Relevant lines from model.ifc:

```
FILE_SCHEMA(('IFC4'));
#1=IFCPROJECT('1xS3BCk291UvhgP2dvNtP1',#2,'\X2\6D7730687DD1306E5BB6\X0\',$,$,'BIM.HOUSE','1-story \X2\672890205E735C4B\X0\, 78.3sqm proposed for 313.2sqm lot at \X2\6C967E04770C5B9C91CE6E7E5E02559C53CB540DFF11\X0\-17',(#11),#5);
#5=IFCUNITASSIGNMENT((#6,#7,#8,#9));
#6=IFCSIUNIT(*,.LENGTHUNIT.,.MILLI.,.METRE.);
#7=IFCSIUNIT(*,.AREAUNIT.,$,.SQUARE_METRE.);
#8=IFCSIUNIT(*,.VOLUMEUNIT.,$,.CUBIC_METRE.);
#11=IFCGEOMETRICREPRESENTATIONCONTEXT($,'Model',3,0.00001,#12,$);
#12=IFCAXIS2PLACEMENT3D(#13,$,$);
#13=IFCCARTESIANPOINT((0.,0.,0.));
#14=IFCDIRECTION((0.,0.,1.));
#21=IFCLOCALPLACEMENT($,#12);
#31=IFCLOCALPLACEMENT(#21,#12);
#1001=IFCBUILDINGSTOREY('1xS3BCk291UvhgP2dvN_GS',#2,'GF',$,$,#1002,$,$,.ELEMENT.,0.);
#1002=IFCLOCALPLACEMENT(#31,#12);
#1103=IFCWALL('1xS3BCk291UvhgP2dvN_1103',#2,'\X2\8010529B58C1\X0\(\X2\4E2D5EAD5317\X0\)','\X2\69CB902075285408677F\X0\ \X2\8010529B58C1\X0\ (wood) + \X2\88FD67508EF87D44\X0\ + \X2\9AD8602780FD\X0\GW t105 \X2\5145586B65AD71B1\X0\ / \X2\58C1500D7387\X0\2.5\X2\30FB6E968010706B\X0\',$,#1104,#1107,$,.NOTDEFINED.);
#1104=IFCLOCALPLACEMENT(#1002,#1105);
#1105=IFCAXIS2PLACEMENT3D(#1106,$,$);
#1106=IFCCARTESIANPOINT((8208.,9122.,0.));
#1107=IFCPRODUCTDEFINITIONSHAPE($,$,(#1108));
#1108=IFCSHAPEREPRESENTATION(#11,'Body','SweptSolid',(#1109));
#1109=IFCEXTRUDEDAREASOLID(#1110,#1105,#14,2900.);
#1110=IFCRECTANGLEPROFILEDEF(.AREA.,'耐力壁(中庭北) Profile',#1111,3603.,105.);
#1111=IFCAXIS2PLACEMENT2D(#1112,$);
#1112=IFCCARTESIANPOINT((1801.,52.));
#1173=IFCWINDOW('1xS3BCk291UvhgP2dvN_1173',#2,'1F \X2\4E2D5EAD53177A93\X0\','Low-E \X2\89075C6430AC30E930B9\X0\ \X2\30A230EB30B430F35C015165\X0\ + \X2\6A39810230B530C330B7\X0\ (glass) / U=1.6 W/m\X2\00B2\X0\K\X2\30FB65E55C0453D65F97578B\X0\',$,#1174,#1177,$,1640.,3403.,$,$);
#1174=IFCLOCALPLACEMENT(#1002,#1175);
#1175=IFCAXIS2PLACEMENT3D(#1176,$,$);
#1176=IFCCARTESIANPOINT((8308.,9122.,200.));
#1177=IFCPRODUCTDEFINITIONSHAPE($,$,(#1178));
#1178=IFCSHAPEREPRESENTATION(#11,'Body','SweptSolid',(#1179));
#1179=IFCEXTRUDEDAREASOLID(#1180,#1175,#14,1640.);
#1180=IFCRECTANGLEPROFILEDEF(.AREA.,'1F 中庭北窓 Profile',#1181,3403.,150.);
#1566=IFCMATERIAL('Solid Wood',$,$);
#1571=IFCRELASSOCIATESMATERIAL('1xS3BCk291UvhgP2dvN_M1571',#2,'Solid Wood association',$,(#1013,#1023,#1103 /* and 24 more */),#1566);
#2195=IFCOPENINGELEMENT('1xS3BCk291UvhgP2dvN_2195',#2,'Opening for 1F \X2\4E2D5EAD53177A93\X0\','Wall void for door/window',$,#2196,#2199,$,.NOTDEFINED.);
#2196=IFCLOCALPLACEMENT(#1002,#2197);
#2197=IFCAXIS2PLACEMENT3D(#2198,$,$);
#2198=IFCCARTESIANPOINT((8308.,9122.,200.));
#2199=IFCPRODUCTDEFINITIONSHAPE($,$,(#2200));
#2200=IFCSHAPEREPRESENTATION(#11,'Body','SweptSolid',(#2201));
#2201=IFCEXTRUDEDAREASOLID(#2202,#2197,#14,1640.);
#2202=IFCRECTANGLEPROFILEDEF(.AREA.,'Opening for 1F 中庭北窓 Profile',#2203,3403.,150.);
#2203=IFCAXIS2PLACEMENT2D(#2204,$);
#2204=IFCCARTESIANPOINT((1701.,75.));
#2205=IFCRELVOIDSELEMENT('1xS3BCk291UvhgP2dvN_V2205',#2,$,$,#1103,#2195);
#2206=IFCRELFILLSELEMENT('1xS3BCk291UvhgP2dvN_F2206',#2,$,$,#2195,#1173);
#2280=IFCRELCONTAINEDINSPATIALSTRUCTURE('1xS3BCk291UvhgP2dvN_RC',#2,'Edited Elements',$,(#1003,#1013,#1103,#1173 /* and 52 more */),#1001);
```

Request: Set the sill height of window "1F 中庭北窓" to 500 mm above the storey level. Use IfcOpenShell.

```python
import numpy as np
import ifcopenshell
import ifcopenshell.api.geometry
import ifcopenshell.geom
import ifcopenshell.util.element
import ifcopenshell.util.placement
import ifcopenshell.util.shape
import ifcopenshell.util.unit

model = ifcopenshell.open("model.ifc")
unit_scale = ifcopenshell.util.unit.calculate_unit_scale(model)

window = model.by_id(1173)
opening = window.FillsVoids[0].RelatingOpeningElement
storey = ifcopenshell.util.element.get_container(window, ifc_class="IfcBuildingStorey")
level = ifcopenshell.util.placement.get_local_placement(storey.ObjectPlacement)[2, 3]

# The opening's origin need not be at the sill, so measure its lowest point.
shape = ifcopenshell.geom.create_shape(ifcopenshell.geom.settings(), opening)
bottom = ifcopenshell.util.shape.get_shape_bottom_elevation(shape, shape.geometry) / unit_scale
dz = level + 500.0 - bottom

shift = np.array([0.0, 0.0, dz])
# The window is not placed relative to its opening, so move both.
for product in (opening, window):
    matrix = ifcopenshell.util.placement.get_local_placement(product.ObjectPlacement)
    matrix[:3, 3] += shift
    ifcopenshell.api.geometry.edit_object_placement(model, product=product, matrix=matrix, is_si=False)

print(f"moved by {dz * unit_scale:+.3f} m")

model.write("model_rev.ifc")
```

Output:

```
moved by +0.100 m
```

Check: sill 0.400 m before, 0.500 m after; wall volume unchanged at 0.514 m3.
